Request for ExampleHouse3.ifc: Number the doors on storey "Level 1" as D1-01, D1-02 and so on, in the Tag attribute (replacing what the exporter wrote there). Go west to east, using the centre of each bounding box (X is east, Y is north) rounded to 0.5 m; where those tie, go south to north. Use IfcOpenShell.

First a look at what the model holds.

```python
import ifcopenshell
import ifcopenshell.util.element
import ifcopenshell.util.placement

model = ifcopenshell.open("ExampleHouse3.ifc")
print(model.schema)
storey = next(s for s in model.by_type("IfcBuildingStorey") if s.Name == "Level 1")
doors = [e for e in ifcopenshell.util.element.get_decomposition(storey) if e.is_a("IfcDoor")]
for e in sorted(doors, key=lambda e: e.id()):
    origin = ifcopenshell.util.placement.get_local_placement(e.ObjectPlacement)[:3, 3]
    print(e.id(), e.Tag, e.Name, origin.round(2) + 0.0, sep=" | ")
```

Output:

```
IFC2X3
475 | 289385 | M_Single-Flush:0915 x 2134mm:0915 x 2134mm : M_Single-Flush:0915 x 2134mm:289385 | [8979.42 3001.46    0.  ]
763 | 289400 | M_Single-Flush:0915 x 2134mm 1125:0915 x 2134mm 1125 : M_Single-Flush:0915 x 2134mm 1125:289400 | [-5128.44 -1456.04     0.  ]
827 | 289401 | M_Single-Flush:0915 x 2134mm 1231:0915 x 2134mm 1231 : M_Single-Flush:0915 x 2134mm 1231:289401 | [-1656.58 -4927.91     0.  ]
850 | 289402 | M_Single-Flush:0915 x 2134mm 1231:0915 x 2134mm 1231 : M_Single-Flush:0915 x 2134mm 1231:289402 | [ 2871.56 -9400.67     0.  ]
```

```python
import ifcopenshell
import ifcopenshell.geom
import ifcopenshell.util.element
import ifcopenshell.util.shape

model = ifcopenshell.open("ExampleHouse3.ifc")
settings = ifcopenshell.geom.settings()
settings.set("use-world-coords", True)


def centre(element):
    shape = ifcopenshell.geom.create_shape(settings, element)
    return ifcopenshell.util.shape.get_bbox_centroid(shape.geometry)


storey = next(s for s in model.by_type("IfcBuildingStorey") if s.Name == "Level 1")
doors = [e for e in ifcopenshell.util.element.get_decomposition(storey) if e.is_a("IfcDoor")]

# Insertion points can sit at a corner or the storey origin, so sort by the geometry (in metres).
centres = {e: centre(e) for e in doors}
doors.sort(key=lambda e: (round(centres[e][0] / 0.5), centres[e][1]))

for i, e in enumerate(doors, start=1):
    number = f"D1-{i:02d}"
    e.Tag = number
    print(e.id(), number)

model.write("ExampleHouse3_updated.ifc")
```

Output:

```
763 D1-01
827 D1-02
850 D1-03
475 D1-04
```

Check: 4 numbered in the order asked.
